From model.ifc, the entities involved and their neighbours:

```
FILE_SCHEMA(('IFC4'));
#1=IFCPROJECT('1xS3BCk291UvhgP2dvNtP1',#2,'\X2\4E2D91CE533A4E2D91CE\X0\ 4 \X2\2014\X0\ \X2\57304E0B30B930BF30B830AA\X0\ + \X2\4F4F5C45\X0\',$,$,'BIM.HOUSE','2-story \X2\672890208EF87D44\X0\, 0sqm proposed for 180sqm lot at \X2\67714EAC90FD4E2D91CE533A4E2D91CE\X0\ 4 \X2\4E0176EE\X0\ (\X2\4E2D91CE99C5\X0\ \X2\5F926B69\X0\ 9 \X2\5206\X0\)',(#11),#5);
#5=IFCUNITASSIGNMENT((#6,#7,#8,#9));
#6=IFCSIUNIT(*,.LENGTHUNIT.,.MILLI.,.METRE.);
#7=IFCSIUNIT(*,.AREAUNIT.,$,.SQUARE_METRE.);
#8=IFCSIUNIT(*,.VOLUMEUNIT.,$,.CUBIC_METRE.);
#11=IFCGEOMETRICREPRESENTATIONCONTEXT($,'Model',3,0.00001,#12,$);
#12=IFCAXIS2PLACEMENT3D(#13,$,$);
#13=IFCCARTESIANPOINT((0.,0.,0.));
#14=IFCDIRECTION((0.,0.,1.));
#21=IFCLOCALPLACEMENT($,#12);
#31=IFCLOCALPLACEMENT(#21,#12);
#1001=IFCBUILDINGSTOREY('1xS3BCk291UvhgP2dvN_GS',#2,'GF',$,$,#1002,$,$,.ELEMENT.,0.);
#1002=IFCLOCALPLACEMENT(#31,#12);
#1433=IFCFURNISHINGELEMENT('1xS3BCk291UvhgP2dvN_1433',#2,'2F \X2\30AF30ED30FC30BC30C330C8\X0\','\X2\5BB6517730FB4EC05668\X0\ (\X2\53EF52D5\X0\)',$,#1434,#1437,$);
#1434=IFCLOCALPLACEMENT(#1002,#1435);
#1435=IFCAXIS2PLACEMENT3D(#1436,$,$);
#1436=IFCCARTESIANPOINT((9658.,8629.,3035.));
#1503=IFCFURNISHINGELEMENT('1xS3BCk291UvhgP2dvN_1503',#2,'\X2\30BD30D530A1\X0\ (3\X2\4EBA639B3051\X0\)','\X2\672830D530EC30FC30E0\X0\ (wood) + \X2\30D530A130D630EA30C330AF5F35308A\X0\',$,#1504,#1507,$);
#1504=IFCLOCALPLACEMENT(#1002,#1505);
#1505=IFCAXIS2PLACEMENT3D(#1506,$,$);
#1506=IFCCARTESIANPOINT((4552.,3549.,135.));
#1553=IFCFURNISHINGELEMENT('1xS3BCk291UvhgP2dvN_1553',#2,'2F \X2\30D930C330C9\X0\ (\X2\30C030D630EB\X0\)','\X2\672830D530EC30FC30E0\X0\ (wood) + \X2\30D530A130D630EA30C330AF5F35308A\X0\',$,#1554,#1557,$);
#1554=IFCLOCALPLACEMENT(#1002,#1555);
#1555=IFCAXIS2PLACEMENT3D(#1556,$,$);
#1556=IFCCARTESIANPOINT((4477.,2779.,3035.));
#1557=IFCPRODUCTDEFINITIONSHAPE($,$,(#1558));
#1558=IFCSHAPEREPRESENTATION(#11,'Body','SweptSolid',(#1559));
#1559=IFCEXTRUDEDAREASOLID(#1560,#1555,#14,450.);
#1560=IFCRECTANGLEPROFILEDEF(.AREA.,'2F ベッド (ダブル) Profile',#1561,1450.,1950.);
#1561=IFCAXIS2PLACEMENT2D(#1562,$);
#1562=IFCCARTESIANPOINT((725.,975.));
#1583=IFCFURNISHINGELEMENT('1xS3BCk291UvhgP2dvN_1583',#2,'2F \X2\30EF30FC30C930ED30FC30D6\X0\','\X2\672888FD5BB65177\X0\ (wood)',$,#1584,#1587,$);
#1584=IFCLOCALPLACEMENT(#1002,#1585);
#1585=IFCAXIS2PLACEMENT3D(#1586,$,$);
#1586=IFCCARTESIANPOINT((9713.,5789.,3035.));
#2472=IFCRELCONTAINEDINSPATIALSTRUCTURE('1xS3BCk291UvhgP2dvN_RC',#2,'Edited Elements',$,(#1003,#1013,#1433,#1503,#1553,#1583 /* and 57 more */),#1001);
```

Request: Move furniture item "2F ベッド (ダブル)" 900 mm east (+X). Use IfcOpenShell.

```python
import ifcopenshell
import ifcopenshell.api.geometry
import ifcopenshell.util.placement

model = ifcopenshell.open("model.ifc")

item = model.by_guid("1xS3BCk291UvhgP2dvN_1553")
matrix = ifcopenshell.util.placement.get_local_placement(item.ObjectPlacement)
matrix[0, 3] += 900.0
ifcopenshell.api.geometry.edit_object_placement(model, product=item, matrix=matrix, is_si=False)

print(ifcopenshell.util.placement.get_local_placement(item.ObjectPlacement).round(3) + 0.0)

model.write("model_v2.ifc")
```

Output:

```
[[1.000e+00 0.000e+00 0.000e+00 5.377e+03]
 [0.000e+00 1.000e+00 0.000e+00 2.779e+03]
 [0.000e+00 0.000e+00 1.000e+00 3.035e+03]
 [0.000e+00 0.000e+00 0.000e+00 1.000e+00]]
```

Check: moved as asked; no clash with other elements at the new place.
